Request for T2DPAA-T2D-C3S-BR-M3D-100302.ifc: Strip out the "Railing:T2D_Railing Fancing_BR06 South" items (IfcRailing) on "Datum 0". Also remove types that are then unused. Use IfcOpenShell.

First a look at what the model holds.

```python
import ifcopenshell
import ifcopenshell.util.element

model = ifcopenshell.open("T2DPAA-T2D-C3S-BR-M3D-100302.ifc")
print(model.schema)
storey = next(s for s in model.by_type("IfcBuildingStorey") if s.Name == "Datum 0")
railings = [e for e in ifcopenshell.util.element.get_decomposition(storey) if e.is_a("IfcRailing")]
seen = {}
for e in railings:
    element_type = ifcopenshell.util.element.get_type(e)
    name = element_type.Name if element_type not in (None, e) else None
    seen[name] = seen.get(name, 0) + 1
for name, count in sorted(seen.items(), key=str):
    print(count, "x", name)
```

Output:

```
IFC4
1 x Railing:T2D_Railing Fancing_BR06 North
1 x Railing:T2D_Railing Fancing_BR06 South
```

```python
import ifcopenshell
import ifcopenshell.api.root
import ifcopenshell.util.element

model = ifcopenshell.open("T2DPAA-T2D-C3S-BR-M3D-100302.ifc")

storey = next(s for s in model.by_type("IfcBuildingStorey") if s.Name == "Datum 0")
railings = [e for e in ifcopenshell.util.element.get_decomposition(storey) if e.is_a("IfcRailing")]
targets = [e for e in railings if (t := ifcopenshell.util.element.get_type(e)) not in (None, e) and t.Name == "Railing:T2D_Railing Fancing_BR06 South"]
types = {ifcopenshell.util.element.get_type(e) for e in targets} - {None, *targets}

for e in targets:
    ifcopenshell.api.root.remove_product(model, product=e)
print(len(targets), "removed")

unused = [t for t in types if not ifcopenshell.util.element.get_types(t)]
for t in unused:
    ifcopenshell.api.root.remove_product(model, product=t)
print(len(unused), "unused types removed")

model.write("T2DPAA-T2D-C3S-BR-M3D-100302_v2.ifc")
```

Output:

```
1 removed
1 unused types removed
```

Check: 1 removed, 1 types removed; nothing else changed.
